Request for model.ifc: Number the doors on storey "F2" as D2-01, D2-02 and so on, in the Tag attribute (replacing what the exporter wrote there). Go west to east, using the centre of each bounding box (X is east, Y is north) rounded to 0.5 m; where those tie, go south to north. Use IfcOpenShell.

First a look at what the model holds.

```python
import ifcopenshell
import ifcopenshell.util.element
import ifcopenshell.util.placement

model = ifcopenshell.open("model.ifc")
print(model.schema)
storey = next(s for s in model.by_type("IfcBuildingStorey") if s.Name == "F2")
doors = [e for e in ifcopenshell.util.element.get_decomposition(storey) if e.is_a("IfcDoor")]
for e in sorted(doors, key=lambda e: e.id()):
    origin = ifcopenshell.util.placement.get_local_placement(e.ObjectPlacement)[:3, 3]
    print(e.id(), e.Tag, e.Name, origin.round(2) + 0.0, sep=" | ")
```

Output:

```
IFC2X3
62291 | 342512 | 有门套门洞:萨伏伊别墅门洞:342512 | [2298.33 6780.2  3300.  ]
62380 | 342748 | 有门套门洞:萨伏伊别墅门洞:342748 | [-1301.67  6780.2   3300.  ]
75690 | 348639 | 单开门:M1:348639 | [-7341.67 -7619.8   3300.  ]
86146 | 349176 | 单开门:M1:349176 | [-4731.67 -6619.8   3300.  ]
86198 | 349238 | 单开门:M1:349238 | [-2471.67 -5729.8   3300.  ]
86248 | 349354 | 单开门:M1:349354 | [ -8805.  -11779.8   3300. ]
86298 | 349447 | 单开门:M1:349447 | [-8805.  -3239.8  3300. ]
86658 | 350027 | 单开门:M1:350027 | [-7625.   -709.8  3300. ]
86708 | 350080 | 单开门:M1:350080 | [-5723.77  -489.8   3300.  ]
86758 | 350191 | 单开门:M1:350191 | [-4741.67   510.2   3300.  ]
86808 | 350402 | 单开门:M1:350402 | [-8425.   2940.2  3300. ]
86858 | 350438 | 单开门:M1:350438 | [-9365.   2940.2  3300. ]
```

```python
import ifcopenshell
import ifcopenshell.geom
import ifcopenshell.util.element
import ifcopenshell.util.shape

model = ifcopenshell.open("model.ifc")
settings = ifcopenshell.geom.settings()
settings.set("use-world-coords", True)


def centre(element):
    shape = ifcopenshell.geom.create_shape(settings, element)
    return ifcopenshell.util.shape.get_bbox_centroid(shape.geometry)


storey = next(s for s in model.by_type("IfcBuildingStorey") if s.Name == "F2")
doors = [e for e in ifcopenshell.util.element.get_decomposition(storey) if e.is_a("IfcDoor")]

# Insertion points can sit at a corner or the storey origin, so sort by the geometry (in metres).
centres = {e: centre(e) for e in doors}
doors.sort(key=lambda e: (round(centres[e][0] / 0.5), centres[e][1]))

for i, e in enumerate(doors, start=1):
    number = f"D2-{i:02d}"
    e.Tag = number
    print(e.id(), number)

model.write("model-out.ifc")
```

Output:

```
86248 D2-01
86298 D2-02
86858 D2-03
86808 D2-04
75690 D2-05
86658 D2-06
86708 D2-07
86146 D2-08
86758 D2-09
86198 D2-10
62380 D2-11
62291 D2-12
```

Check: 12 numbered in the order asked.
